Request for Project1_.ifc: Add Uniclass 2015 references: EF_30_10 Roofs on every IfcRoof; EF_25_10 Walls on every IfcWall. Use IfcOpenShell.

First a look at what the model holds.

```python
import ifcopenshell

model = ifcopenshell.open("Project1_.ifc")
print(model.schema)
print("classifications:", [c.Name for c in model.by_type("IfcClassification")])
for ifc_class in ("IfcDoor", "IfcRoof", "IfcStair", "IfcWall", "IfcWindow"):
    print(ifc_class, len(model.by_type(ifc_class)))
```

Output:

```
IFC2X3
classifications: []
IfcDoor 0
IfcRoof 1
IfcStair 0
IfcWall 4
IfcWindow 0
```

```python
import ifcopenshell
import ifcopenshell.api.classification

model = ifcopenshell.open("Project1_.ifc")

# IFC2X3 requires Source and Edition and has no link from the project to the system.
system = model.create_entity("IfcClassification", Source="NBS", Edition="2015", Name="Uniclass 2015")

codes = {
    "IfcRoof": ("EF_30_10", "Roofs"),
    "IfcWall": ("EF_25_10", "Walls"),
}
for ifc_class, (code, name) in codes.items():
    products = model.by_type(ifc_class)
    ifcopenshell.api.classification.add_reference(
        model, products=products, classification=system, identification=code, name=name
    )
    print(code, len(products))

model.write("Project1__v2.ifc")
```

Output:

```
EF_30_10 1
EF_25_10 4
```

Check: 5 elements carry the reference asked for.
